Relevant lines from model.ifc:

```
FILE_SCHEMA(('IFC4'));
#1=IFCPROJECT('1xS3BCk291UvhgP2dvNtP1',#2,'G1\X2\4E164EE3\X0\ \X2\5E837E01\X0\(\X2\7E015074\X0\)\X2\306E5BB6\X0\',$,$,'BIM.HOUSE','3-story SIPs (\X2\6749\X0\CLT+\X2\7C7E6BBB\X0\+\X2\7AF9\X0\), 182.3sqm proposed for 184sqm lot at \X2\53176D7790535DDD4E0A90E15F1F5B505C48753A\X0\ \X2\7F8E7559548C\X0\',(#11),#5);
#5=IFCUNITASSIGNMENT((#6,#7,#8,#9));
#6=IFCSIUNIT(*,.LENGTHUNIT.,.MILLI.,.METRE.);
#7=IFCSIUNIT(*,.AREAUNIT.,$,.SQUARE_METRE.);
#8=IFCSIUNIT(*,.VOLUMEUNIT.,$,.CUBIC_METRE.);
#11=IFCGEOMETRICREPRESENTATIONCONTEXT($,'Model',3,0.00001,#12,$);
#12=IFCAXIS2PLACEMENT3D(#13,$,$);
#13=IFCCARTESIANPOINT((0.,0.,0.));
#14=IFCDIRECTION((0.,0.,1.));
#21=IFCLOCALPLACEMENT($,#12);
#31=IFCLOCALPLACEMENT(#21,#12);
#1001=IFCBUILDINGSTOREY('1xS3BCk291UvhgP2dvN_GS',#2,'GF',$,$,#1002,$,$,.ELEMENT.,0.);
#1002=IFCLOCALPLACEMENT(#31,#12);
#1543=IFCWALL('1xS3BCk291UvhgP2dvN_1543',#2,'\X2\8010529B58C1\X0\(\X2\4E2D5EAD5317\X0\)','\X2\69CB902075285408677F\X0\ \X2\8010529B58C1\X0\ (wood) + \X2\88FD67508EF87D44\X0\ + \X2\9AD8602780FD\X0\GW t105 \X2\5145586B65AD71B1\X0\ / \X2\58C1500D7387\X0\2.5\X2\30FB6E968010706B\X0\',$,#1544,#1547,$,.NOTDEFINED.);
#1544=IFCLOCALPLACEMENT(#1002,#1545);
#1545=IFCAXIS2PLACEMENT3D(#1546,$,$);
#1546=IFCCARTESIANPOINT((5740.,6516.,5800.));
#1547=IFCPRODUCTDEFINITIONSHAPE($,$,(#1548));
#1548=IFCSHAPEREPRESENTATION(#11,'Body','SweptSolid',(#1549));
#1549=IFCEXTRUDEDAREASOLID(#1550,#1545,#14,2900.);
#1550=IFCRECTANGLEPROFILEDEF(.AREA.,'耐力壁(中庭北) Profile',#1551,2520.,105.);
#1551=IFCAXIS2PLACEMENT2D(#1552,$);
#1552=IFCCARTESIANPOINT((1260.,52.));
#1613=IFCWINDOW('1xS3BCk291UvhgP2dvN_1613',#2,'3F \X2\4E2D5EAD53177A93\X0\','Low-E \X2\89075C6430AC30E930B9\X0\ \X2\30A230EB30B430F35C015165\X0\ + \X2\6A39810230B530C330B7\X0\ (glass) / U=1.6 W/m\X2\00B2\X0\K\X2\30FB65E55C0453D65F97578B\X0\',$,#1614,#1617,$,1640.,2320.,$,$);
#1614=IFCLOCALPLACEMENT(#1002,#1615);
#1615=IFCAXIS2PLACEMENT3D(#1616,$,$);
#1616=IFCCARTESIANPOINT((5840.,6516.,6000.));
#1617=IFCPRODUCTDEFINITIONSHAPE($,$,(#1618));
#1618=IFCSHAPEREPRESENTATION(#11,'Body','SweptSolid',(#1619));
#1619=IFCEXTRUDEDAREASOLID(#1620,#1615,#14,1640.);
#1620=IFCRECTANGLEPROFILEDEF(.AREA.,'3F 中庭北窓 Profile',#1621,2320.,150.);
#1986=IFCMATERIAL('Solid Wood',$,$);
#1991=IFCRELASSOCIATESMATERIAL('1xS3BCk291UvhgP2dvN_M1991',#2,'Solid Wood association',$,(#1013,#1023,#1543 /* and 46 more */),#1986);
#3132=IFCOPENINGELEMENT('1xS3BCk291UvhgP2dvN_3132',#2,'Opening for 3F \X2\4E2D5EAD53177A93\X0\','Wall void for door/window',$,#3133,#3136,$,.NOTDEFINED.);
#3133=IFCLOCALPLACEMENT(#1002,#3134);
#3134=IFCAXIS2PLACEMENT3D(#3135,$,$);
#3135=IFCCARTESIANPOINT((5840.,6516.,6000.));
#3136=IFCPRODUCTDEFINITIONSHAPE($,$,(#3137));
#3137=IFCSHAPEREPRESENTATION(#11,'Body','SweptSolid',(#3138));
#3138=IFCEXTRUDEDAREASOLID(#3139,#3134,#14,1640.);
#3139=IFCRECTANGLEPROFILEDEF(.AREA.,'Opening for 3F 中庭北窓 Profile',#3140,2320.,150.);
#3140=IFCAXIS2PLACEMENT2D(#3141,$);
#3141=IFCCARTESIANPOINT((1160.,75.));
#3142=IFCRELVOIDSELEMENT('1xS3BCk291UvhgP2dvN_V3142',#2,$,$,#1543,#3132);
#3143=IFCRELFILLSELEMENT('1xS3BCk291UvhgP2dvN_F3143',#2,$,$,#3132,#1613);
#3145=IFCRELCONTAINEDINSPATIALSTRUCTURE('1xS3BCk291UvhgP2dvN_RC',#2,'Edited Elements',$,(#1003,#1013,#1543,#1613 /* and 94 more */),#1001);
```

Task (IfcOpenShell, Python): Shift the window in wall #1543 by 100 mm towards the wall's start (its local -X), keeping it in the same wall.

```python
import ifcopenshell
import ifcopenshell.api.geometry
import ifcopenshell.util.placement
import ifcopenshell.util.unit

model = ifcopenshell.open("model.ifc")
unit_scale = ifcopenshell.util.unit.calculate_unit_scale(model)

window = model.by_guid("1xS3BCk291UvhgP2dvN_1613")
opening = window.FillsVoids[0].RelatingOpeningElement
wall = opening.VoidsElements[0].RelatingBuildingElement

wall_matrix = ifcopenshell.util.placement.get_local_placement(wall.ObjectPlacement)
shift = wall_matrix[:3, 0] * -0.1 / unit_scale
before = ifcopenshell.util.placement.get_local_placement(window.ObjectPlacement)[:3, 3].copy()

# The window is not placed relative to its opening, so move both.
for product in (opening, window):
    matrix = ifcopenshell.util.placement.get_local_placement(product.ObjectPlacement)
    matrix[:3, 3] += shift
    ifcopenshell.api.geometry.edit_object_placement(model, product=product, matrix=matrix, is_si=False)

after = ifcopenshell.util.placement.get_local_placement(window.ObjectPlacement)[:3, 3]
print("window moved by", (after - before).round(3) + 0.0)

model.write("model-out.ifc")
```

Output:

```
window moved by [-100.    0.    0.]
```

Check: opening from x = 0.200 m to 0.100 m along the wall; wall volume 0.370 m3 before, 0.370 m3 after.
